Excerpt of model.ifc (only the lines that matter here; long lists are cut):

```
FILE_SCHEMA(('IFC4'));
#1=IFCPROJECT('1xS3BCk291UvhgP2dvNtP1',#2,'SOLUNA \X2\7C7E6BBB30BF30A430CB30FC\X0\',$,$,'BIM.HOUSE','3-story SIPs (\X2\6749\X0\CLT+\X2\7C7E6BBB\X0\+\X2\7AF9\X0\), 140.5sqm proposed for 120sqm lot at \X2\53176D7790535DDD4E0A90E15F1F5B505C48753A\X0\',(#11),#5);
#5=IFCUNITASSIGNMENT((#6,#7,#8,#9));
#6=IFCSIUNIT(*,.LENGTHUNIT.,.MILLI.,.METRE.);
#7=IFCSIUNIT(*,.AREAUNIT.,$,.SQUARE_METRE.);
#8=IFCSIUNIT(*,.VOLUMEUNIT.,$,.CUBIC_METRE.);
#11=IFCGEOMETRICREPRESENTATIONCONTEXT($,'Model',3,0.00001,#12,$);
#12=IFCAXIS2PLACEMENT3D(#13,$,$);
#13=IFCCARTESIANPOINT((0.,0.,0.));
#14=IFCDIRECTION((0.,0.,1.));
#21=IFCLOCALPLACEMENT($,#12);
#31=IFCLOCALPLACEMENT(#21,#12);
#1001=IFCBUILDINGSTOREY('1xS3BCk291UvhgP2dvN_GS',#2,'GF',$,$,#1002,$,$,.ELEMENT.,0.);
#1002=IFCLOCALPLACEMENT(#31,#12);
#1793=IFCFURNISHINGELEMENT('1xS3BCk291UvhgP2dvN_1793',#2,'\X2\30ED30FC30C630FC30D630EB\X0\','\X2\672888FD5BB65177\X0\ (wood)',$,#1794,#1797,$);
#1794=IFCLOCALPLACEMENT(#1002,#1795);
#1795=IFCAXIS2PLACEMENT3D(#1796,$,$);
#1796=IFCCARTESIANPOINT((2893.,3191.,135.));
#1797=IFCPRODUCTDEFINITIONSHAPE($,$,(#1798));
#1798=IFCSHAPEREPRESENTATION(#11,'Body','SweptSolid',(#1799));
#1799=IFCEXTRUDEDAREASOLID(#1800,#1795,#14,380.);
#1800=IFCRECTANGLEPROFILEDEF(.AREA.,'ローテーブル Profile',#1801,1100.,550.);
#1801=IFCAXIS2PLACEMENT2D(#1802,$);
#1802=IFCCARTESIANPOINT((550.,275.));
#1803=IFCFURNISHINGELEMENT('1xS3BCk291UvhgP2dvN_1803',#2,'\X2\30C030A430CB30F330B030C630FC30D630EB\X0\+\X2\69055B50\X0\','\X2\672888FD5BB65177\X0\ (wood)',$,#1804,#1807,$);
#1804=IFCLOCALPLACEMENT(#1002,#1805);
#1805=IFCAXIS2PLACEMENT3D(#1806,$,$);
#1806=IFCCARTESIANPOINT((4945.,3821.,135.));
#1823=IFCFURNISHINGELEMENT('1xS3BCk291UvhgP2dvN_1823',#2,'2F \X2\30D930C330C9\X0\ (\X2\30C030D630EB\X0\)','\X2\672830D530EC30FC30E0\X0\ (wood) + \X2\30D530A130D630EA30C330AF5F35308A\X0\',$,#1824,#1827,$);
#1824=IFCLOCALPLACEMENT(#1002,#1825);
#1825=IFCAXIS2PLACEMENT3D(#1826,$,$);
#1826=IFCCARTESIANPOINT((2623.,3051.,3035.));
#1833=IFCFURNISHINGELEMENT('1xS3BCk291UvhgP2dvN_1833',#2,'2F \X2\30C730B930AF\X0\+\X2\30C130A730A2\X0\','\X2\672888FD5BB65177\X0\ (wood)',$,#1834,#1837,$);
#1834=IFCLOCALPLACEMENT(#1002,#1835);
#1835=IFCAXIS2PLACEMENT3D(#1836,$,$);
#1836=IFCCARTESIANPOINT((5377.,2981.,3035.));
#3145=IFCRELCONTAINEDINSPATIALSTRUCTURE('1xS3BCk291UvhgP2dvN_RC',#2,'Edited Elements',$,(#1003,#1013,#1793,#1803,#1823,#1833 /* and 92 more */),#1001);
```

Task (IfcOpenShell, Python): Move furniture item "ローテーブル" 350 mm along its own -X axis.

```python
import ifcopenshell
import ifcopenshell.api.geometry
import ifcopenshell.util.placement

model = ifcopenshell.open("model.ifc")

item = model.by_id(1793)
matrix = ifcopenshell.util.placement.get_local_placement(item.ObjectPlacement)
matrix[:3, 3] -= matrix[:3, 0] * 350.0
ifcopenshell.api.geometry.edit_object_placement(model, product=item, matrix=matrix, is_si=False)

print(ifcopenshell.util.placement.get_local_placement(item.ObjectPlacement).round(3) + 0.0)

model.write("model_edited.ifc")
```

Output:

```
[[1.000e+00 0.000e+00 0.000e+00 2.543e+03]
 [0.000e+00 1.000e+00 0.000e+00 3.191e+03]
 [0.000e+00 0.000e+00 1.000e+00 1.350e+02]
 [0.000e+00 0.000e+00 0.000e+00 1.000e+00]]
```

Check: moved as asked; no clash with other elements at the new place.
